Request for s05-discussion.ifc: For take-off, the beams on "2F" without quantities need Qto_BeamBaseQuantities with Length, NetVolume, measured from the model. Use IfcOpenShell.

First a look at what the model holds.

```python
import ifcopenshell
import ifcopenshell.util.element
import ifcopenshell.util.unit

model = ifcopenshell.open("s05-discussion.ifc")
print(model.schema)
for unit_type in ("LENGTHUNIT", "AREAUNIT", "VOLUMEUNIT"):
    print(unit_type, ifcopenshell.util.unit.calculate_unit_scale(model, unit_type))
storey = next(s for s in model.by_type("IfcBuildingStorey") if s.Name == "2F")
beams = [e for e in ifcopenshell.util.element.get_decomposition(storey) if e.is_a("IfcBeam")]
for e in sorted(beams, key=lambda e: e.id()):
    print(e.id(), e.is_a(), e.Name, list(ifcopenshell.util.element.get_psets(e, qtos_only=True)), sep=" | ")
```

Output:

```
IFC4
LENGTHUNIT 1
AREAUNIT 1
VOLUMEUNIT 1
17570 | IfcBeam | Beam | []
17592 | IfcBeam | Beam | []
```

```python
import ifcopenshell
import ifcopenshell.api.pset
import ifcopenshell.geom
import ifcopenshell.util.element
import ifcopenshell.util.shape
import ifcopenshell.util.unit

model = ifcopenshell.open("s05-discussion.ifc")
unit_scale = ifcopenshell.util.unit.calculate_unit_scale(model)
volume_scale = ifcopenshell.util.unit.calculate_unit_scale(model, "VOLUMEUNIT")
settings = ifcopenshell.geom.settings()

storey = next(s for s in model.by_type("IfcBuildingStorey") if s.Name == "2F")
beams = [e for e in ifcopenshell.util.element.get_decomposition(storey) if e.is_a("IfcBeam")]

for e in sorted(beams, key=lambda e: e.id()):
    if ifcopenshell.util.element.get_psets(e, qtos_only=True, should_inherit=False):
        continue
    # Geometry comes back in metres, in the element's own axes.
    shape = ifcopenshell.geom.create_shape(settings, e)
    values = {
        "Length": ifcopenshell.util.shape.get_max_xyz(shape.geometry) / unit_scale,
        "NetVolume": ifcopenshell.util.shape.get_volume(shape.geometry) / volume_scale,
    }
    qto = ifcopenshell.api.pset.add_qto(model, product=e, name="Qto_BeamBaseQuantities")
    ifcopenshell.api.pset.edit_qto(model, qto=qto, properties=values)
    print(e.id(), {k: round(v, 3) for k, v in values.items()})

model.write("s05-discussion_v2.ifc")
```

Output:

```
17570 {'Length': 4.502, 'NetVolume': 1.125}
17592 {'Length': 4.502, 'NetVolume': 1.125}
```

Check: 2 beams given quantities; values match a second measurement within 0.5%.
